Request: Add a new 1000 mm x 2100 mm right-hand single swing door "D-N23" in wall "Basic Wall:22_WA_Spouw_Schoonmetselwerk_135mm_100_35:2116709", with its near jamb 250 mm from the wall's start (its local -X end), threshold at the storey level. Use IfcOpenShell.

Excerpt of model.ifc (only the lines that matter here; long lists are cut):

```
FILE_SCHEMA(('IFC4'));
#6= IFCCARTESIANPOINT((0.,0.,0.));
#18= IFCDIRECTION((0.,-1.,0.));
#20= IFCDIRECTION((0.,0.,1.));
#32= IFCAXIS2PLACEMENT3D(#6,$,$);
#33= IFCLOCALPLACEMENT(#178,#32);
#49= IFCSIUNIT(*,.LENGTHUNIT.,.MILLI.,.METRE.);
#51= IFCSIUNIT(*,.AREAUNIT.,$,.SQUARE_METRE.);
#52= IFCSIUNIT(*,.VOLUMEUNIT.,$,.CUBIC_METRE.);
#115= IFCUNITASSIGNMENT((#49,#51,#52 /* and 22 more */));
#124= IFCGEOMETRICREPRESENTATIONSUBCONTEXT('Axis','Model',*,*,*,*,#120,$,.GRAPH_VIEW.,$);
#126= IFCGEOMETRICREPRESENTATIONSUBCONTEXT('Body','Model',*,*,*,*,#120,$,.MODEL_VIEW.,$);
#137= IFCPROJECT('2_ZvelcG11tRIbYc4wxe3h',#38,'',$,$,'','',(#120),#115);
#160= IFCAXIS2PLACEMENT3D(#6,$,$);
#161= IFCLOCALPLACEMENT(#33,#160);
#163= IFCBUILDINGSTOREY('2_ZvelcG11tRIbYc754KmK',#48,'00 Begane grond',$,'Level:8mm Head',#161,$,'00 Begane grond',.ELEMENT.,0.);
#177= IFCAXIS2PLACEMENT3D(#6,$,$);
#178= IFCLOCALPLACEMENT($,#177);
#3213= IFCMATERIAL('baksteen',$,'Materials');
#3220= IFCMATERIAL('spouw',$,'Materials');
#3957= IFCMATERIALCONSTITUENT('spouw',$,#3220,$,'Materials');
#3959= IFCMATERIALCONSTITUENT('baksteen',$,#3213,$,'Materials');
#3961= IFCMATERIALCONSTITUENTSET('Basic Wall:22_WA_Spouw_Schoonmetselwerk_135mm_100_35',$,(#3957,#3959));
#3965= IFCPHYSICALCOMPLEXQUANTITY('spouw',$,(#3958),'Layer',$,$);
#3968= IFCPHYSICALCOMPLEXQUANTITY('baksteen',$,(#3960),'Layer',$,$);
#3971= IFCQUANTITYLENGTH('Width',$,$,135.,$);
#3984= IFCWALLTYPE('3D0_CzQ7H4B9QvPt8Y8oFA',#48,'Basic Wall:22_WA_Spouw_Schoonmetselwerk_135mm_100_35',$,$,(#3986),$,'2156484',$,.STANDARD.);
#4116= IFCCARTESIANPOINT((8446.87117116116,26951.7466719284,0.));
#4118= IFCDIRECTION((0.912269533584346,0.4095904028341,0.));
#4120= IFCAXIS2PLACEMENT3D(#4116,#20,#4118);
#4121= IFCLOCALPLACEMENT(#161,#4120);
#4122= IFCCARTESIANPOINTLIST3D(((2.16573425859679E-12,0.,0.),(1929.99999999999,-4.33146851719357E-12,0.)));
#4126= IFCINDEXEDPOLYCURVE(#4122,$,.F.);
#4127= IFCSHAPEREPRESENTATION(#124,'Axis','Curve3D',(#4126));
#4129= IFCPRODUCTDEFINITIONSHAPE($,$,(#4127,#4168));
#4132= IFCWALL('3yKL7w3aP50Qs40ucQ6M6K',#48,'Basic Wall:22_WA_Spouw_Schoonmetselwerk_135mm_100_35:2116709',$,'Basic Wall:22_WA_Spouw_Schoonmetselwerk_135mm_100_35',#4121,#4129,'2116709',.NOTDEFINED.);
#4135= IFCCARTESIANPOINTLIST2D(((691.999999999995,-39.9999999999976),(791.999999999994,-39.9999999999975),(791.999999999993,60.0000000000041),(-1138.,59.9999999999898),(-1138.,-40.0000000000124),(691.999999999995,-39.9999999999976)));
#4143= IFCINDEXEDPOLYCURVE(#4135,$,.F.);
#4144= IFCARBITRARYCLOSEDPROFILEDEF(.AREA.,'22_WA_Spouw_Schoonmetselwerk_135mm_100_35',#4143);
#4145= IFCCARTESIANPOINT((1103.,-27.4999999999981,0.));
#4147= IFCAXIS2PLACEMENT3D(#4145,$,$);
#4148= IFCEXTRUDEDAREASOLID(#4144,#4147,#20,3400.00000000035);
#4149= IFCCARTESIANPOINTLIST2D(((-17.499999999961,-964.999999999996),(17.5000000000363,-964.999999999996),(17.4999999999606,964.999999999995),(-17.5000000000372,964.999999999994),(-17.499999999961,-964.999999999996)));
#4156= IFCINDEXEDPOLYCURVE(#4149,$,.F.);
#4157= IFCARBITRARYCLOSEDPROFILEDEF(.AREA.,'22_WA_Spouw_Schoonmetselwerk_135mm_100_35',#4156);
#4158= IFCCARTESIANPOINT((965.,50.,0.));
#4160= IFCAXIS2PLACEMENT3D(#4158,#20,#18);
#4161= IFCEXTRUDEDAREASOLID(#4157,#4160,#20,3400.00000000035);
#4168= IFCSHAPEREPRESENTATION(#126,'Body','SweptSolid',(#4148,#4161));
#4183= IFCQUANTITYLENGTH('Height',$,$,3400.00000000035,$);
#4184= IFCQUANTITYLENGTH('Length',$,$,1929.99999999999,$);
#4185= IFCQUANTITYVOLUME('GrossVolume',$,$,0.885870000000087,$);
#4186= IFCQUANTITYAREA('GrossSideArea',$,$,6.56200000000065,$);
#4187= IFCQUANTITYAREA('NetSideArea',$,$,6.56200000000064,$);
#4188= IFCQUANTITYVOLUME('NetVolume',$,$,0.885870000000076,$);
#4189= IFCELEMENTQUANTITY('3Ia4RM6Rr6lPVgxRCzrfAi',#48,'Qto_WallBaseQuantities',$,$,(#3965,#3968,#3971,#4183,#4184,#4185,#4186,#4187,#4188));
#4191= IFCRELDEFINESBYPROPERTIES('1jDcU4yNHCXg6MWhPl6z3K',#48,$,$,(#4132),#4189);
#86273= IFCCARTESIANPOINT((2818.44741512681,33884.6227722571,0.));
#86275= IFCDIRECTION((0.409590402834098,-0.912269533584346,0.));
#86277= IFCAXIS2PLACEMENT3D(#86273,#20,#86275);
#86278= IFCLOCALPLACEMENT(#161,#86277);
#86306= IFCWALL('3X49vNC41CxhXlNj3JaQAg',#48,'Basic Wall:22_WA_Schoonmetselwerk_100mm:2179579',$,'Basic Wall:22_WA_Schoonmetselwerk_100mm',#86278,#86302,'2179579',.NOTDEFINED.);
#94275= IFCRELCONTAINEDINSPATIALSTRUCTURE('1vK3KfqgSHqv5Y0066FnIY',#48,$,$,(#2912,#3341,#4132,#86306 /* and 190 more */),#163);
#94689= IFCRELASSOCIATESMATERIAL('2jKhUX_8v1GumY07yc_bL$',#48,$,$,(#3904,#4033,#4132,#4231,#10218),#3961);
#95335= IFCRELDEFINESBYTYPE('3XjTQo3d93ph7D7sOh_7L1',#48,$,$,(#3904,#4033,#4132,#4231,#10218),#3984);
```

```python
import numpy as np
import ifcopenshell
import ifcopenshell.api.feature
import ifcopenshell.api.geometry
import ifcopenshell.api.pset
import ifcopenshell.api.root
import ifcopenshell.api.spatial
import ifcopenshell.geom
import ifcopenshell.util.element
import ifcopenshell.util.placement
import ifcopenshell.util.representation
import ifcopenshell.util.shape
import ifcopenshell.util.unit

model = ifcopenshell.open("model.ifc")
unit_scale = ifcopenshell.util.unit.calculate_unit_scale(model)
area_scale = ifcopenshell.util.unit.calculate_unit_scale(model, "AREAUNIT")
volume_scale = ifcopenshell.util.unit.calculate_unit_scale(model, "VOLUMEUNIT")
settings = ifcopenshell.geom.settings()


def volume(element):
    """Net volume in cubic metres, openings subtracted."""
    shape = ifcopenshell.geom.create_shape(settings, element)
    return ifcopenshell.util.shape.get_volume(shape.geometry)


wall = model.by_guid("3yKL7w3aP50Qs40ucQ6M6K")
storey = ifcopenshell.util.element.get_container(wall, ifc_class="IfcBuildingStorey")
context = ifcopenshell.util.representation.get_context(model, "Model", "Body", "MODEL_VIEW")
before = volume(wall)

width, height, from_end, sill = 1, 2.1, 0.25, 0.0  # metres

# The wall runs along its own X axis, and the end named is its -X end.
wall_shape = ifcopenshell.geom.create_shape(settings, wall)
x, y, z = ifcopenshell.util.shape.get_vertices(wall_shape.geometry).T
start = x.min() + from_end
face, thickness = float(y.min()), float(y.max() - y.min())
wall_matrix = ifcopenshell.util.placement.get_local_placement(wall.ObjectPlacement)
level = ifcopenshell.util.placement.get_local_placement(storey.ObjectPlacement)[2, 3]


def in_wall(x, y):
    """Placement at x, y metres in the wall's axes, at sill height."""
    matrix = wall_matrix.copy()
    matrix[:, 3] = wall_matrix @ np.array([x / unit_scale, y / unit_scale, 0.0, 1.0])
    matrix[2, 3] = level + sill / unit_scale
    return matrix


# Opening: a box that overshoots both wall faces by 50 mm.
opening = ifcopenshell.api.root.create_entity(model, ifc_class="IfcOpeningElement", predefined_type="OPENING")
box = ifcopenshell.api.geometry.add_wall_representation(
    model, context=context, length=width, height=height, thickness=thickness + 0.1
)
ifcopenshell.api.geometry.assign_representation(model, product=opening, representation=box)
ifcopenshell.api.geometry.edit_object_placement(model, product=opening, matrix=in_wall(start, face - 0.05), is_si=False)
ifcopenshell.api.feature.add_feature(model, feature=opening, element=wall)

door = ifcopenshell.api.root.create_entity(model, ifc_class="IfcDoor", name="D-N23", predefined_type="DOOR")
door.OverallWidth, door.OverallHeight = width / unit_scale, height / unit_scale
door.OperationType = "SINGLE_SWING_RIGHT"
body = ifcopenshell.api.geometry.add_door_representation(
    model,
    context=context,
    overall_width=door.OverallWidth,
    overall_height=door.OverallHeight,
    operation_type="SINGLE_SWING_RIGHT",
    lining_properties={"LiningDepth": thickness / unit_scale, "ThresholdDepth": thickness / unit_scale},
)
ifcopenshell.api.geometry.assign_representation(model, product=door, representation=body)
ifcopenshell.api.spatial.assign_container(model, products=[door], relating_structure=storey)
ifcopenshell.api.feature.add_filling(model, opening=opening, element=door)

# The lining spans the wall, so the door starts at the wall face.
ifcopenshell.api.geometry.edit_object_placement(model, product=door, matrix=in_wall(start, face), is_si=False)

after = volume(wall)

# Update the wall's stored quantities.
qto = model.by_id(ifcopenshell.util.element.get_pset(wall, "Qto_WallBaseQuantities", should_inherit=False)["id"])
ifcopenshell.api.pset.edit_qto(model, qto=qto, properties={
    "NetSideArea": after / thickness / area_scale,
    "NetVolume": after / volume_scale,
})

print(f"wall volume {before:.3f} -> {after:.3f} m3")

model.write("model_edited.ifc")
```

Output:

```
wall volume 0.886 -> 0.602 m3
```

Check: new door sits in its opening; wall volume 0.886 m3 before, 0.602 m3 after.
